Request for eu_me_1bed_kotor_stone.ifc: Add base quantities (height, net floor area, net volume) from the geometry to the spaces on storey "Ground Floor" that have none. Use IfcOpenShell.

First a look at what the model holds.

```python
import ifcopenshell
import ifcopenshell.util.element
import ifcopenshell.util.unit

model = ifcopenshell.open("eu_me_1bed_kotor_stone.ifc")
print(model.schema)
for unit_type in ("LENGTHUNIT", "AREAUNIT", "VOLUMEUNIT"):
    print(unit_type, ifcopenshell.util.unit.calculate_unit_scale(model, unit_type))
storey = next(s for s in model.by_type("IfcBuildingStorey") if s.Name == "Ground Floor")
spaces = [e for e in ifcopenshell.util.element.get_decomposition(storey) if e.is_a("IfcSpace")]
for e in sorted(spaces, key=lambda e: e.id()):
    print(e.id(), e.is_a(), e.Name, list(ifcopenshell.util.element.get_psets(e, qtos_only=True)), sep=" | ")
```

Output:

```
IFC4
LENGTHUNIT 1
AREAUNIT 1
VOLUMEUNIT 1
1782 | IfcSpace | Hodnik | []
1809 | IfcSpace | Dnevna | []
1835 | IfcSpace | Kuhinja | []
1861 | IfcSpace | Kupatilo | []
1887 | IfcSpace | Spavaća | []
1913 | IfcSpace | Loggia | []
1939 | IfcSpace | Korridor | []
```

```python
import ifcopenshell
import ifcopenshell.api.pset
import ifcopenshell.geom
import ifcopenshell.util.element
import ifcopenshell.util.shape
import ifcopenshell.util.unit

model = ifcopenshell.open("eu_me_1bed_kotor_stone.ifc")
unit_scale = ifcopenshell.util.unit.calculate_unit_scale(model)
area_scale = ifcopenshell.util.unit.calculate_unit_scale(model, "AREAUNIT")
volume_scale = ifcopenshell.util.unit.calculate_unit_scale(model, "VOLUMEUNIT")
settings = ifcopenshell.geom.settings()

storey = next(s for s in model.by_type("IfcBuildingStorey") if s.Name == "Ground Floor")
spaces = [e for e in ifcopenshell.util.element.get_decomposition(storey) if e.is_a("IfcSpace")]

for e in sorted(spaces, key=lambda e: e.id()):
    if ifcopenshell.util.element.get_psets(e, qtos_only=True, should_inherit=False):
        continue
    # Geometry comes back in metres, in the element's own axes.
    shape = ifcopenshell.geom.create_shape(settings, e)
    values = {
        "Height": ifcopenshell.util.shape.get_z(shape.geometry) / unit_scale,
        "NetFloorArea": ifcopenshell.util.shape.get_footprint_area(shape.geometry) / area_scale,
        "NetVolume": ifcopenshell.util.shape.get_volume(shape.geometry) / volume_scale,
    }
    qto = ifcopenshell.api.pset.add_qto(model, product=e, name="Qto_SpaceBaseQuantities")
    ifcopenshell.api.pset.edit_qto(model, qto=qto, properties=values)
    print(e.id(), {k: round(v, 3) for k, v in values.items()})

model.write("eu_me_1bed_kotor_stone_rev.ifc")
```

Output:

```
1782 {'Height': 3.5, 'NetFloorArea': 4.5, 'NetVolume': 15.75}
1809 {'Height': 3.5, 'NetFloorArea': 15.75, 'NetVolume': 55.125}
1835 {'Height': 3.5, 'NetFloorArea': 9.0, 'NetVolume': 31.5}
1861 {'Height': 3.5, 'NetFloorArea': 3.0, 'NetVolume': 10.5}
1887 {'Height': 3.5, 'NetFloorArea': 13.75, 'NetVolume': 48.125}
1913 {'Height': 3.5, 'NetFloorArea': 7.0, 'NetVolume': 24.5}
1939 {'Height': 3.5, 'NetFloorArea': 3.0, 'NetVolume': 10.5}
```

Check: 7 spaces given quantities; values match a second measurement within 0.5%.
